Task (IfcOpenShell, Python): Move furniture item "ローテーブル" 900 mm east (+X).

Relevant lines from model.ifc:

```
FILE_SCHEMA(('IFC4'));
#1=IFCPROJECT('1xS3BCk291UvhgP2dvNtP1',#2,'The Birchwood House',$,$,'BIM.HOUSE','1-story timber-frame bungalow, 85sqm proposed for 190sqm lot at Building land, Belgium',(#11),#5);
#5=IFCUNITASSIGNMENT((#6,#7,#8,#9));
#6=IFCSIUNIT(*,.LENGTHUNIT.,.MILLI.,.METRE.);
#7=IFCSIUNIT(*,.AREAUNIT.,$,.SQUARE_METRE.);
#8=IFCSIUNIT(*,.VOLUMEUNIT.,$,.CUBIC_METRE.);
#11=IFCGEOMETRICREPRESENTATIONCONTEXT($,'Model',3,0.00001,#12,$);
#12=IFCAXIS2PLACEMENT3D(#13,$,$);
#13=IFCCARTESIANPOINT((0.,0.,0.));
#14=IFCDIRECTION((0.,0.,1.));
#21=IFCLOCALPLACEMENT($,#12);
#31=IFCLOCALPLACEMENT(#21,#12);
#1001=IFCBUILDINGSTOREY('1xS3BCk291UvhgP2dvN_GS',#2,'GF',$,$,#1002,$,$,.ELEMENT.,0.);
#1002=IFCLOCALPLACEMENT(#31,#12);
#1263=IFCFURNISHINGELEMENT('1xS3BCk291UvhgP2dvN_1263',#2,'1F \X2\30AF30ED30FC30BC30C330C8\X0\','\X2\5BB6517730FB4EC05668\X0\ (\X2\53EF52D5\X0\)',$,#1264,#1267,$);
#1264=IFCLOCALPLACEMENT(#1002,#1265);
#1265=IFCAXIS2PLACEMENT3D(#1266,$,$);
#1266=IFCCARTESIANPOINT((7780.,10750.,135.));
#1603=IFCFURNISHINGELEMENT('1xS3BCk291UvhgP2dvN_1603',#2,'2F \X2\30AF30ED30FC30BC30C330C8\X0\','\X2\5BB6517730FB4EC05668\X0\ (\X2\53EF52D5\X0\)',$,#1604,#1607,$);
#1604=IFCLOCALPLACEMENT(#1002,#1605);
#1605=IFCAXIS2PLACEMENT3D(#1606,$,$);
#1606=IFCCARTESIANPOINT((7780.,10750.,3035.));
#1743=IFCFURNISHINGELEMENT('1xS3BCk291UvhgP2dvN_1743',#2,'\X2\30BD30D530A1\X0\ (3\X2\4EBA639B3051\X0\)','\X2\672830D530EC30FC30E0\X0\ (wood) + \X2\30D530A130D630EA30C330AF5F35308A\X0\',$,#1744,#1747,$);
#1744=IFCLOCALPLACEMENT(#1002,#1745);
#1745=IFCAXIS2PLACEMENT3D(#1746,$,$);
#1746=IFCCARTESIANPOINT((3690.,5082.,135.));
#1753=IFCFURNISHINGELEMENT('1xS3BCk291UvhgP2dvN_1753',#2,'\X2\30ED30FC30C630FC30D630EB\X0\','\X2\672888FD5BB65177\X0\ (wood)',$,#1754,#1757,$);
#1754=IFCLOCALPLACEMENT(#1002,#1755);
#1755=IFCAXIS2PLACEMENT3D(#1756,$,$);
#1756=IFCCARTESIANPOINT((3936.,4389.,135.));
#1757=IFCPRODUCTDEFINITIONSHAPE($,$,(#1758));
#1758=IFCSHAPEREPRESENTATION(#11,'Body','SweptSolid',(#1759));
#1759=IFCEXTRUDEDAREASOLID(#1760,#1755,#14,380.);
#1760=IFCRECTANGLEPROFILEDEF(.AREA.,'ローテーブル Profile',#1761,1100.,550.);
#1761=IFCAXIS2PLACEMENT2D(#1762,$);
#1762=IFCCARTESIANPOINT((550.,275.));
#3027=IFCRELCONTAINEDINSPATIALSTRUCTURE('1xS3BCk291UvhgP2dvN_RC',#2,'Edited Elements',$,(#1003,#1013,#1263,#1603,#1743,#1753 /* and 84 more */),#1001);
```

```python
import ifcopenshell
import ifcopenshell.api.geometry
import ifcopenshell.util.placement

model = ifcopenshell.open("model.ifc")

item = model.by_guid("1xS3BCk291UvhgP2dvN_1753")
matrix = ifcopenshell.util.placement.get_local_placement(item.ObjectPlacement)
matrix[0, 3] += 900.0
ifcopenshell.api.geometry.edit_object_placement(model, product=item, matrix=matrix, is_si=False)

print(ifcopenshell.util.placement.get_local_placement(item.ObjectPlacement).round(3) + 0.0)

model.write("model_edited.ifc")
```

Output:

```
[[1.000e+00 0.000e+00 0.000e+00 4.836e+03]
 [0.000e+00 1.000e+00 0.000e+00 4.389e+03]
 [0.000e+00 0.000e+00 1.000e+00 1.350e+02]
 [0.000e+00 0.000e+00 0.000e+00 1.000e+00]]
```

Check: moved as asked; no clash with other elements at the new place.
